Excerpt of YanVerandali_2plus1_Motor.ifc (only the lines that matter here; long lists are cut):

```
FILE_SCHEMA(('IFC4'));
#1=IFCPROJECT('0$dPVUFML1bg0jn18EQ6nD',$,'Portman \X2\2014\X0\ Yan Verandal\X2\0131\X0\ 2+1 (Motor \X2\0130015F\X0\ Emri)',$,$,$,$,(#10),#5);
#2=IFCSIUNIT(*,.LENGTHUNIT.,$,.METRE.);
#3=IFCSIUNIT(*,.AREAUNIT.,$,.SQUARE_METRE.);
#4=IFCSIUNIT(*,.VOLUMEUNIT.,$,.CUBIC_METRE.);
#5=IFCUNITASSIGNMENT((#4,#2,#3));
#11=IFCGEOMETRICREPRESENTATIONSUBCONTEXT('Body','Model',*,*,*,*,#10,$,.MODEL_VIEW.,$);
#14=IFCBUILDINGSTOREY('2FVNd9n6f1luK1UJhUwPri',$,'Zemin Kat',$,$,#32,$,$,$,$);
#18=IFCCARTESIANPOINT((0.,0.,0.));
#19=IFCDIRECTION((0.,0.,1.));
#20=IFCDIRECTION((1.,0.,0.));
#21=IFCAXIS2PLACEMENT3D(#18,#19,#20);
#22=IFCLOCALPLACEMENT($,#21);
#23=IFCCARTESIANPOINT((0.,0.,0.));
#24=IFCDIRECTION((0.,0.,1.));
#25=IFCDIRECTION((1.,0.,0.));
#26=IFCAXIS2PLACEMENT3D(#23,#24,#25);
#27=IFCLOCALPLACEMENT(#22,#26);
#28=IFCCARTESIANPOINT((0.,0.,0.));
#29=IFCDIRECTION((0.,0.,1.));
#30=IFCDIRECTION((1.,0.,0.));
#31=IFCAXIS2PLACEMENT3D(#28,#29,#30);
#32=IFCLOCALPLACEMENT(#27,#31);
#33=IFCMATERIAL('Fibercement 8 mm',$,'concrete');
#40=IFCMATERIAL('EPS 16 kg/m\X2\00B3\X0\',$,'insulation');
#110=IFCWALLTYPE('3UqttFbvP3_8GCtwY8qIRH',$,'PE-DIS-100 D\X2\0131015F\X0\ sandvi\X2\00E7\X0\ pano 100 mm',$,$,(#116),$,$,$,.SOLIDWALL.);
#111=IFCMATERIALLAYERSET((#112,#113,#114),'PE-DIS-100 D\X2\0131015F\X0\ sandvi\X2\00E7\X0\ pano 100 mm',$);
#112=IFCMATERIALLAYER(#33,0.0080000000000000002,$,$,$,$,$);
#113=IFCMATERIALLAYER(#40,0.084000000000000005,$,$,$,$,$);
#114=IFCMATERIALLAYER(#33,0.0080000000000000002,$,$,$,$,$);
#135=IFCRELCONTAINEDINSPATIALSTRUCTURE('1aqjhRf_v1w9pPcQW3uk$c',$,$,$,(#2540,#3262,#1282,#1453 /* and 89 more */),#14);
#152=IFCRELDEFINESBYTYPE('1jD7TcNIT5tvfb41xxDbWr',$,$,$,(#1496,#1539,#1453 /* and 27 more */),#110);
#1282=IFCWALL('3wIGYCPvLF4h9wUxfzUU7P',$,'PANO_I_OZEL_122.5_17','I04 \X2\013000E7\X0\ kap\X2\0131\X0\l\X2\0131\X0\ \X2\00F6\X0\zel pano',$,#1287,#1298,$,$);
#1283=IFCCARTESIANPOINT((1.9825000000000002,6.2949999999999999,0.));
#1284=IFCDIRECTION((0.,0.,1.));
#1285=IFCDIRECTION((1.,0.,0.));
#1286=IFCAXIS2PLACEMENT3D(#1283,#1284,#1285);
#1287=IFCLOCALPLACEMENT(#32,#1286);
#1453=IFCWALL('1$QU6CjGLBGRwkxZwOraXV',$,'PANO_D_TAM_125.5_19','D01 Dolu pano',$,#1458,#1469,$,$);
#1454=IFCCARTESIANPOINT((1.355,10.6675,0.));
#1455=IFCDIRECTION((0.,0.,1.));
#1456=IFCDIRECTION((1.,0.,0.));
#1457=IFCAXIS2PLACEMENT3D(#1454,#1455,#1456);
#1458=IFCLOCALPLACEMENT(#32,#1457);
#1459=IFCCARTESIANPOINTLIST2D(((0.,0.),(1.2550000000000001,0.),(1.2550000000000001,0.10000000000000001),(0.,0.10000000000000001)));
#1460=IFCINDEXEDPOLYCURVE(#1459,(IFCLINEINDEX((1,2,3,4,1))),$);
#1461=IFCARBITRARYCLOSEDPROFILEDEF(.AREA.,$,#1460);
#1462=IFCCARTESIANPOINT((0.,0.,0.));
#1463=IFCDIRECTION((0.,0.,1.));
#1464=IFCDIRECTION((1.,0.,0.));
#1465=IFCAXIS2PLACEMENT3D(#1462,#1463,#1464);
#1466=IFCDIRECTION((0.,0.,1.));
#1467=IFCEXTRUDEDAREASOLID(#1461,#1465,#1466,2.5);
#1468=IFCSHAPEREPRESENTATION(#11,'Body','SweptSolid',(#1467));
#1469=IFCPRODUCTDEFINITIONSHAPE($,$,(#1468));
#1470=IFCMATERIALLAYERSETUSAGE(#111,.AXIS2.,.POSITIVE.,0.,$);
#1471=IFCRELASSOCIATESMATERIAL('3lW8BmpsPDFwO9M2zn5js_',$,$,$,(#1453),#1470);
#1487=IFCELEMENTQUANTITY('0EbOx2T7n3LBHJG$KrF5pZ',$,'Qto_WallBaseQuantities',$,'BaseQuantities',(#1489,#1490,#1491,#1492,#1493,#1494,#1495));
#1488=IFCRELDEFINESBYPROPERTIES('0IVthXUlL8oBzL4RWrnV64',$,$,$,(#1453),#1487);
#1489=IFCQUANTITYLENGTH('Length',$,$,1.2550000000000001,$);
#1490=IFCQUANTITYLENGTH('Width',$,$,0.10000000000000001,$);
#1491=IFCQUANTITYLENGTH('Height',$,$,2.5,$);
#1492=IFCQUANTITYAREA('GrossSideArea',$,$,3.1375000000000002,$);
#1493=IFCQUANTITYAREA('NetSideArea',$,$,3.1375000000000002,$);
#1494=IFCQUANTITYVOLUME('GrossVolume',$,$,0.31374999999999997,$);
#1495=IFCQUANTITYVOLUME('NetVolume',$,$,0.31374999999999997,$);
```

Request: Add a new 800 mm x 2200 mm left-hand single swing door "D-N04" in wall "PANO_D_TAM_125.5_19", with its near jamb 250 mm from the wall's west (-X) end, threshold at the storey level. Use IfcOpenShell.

```python
import numpy as np
import ifcopenshell
import ifcopenshell.api.feature
import ifcopenshell.api.geometry
import ifcopenshell.api.pset
import ifcopenshell.api.root
import ifcopenshell.api.spatial
import ifcopenshell.geom
import ifcopenshell.util.element
import ifcopenshell.util.placement
import ifcopenshell.util.representation
import ifcopenshell.util.shape
import ifcopenshell.util.unit

model = ifcopenshell.open("YanVerandali_2plus1_Motor.ifc")
unit_scale = ifcopenshell.util.unit.calculate_unit_scale(model)
area_scale = ifcopenshell.util.unit.calculate_unit_scale(model, "AREAUNIT")
volume_scale = ifcopenshell.util.unit.calculate_unit_scale(model, "VOLUMEUNIT")
settings = ifcopenshell.geom.settings()


def volume(element):
    """Net volume in cubic metres, openings subtracted."""
    shape = ifcopenshell.geom.create_shape(settings, element)
    return ifcopenshell.util.shape.get_volume(shape.geometry)


wall = model.by_guid("1$QU6CjGLBGRwkxZwOraXV")
storey = ifcopenshell.util.element.get_container(wall, ifc_class="IfcBuildingStorey")
context = ifcopenshell.util.representation.get_context(model, "Model", "Body", "MODEL_VIEW")
before = volume(wall)

width, height, from_end, sill = 0.8, 2.2, 0.25, 0.0  # metres

# The wall runs along its own X axis, and the end named is its -X end.
wall_shape = ifcopenshell.geom.create_shape(settings, wall)
x, y, z = ifcopenshell.util.shape.get_vertices(wall_shape.geometry).T
start = x.min() + from_end
face, thickness = float(y.min()), float(y.max() - y.min())
wall_matrix = ifcopenshell.util.placement.get_local_placement(wall.ObjectPlacement)
level = ifcopenshell.util.placement.get_local_placement(storey.ObjectPlacement)[2, 3]


def in_wall(x, y):
    """Placement at x, y metres in the wall's axes, at sill height."""
    matrix = wall_matrix.copy()
    matrix[:, 3] = wall_matrix @ np.array([x / unit_scale, y / unit_scale, 0.0, 1.0])
    matrix[2, 3] = level + sill / unit_scale
    return matrix


# Opening: a box that overshoots both wall faces by 50 mm.
opening = ifcopenshell.api.root.create_entity(model, ifc_class="IfcOpeningElement", predefined_type="OPENING")
box = ifcopenshell.api.geometry.add_wall_representation(
    model, context=context, length=width, height=height, thickness=thickness + 0.1
)
ifcopenshell.api.geometry.assign_representation(model, product=opening, representation=box)
ifcopenshell.api.geometry.edit_object_placement(model, product=opening, matrix=in_wall(start, face - 0.05), is_si=False)
ifcopenshell.api.feature.add_feature(model, feature=opening, element=wall)

door = ifcopenshell.api.root.create_entity(model, ifc_class="IfcDoor", name="D-N04", predefined_type="DOOR")
door.OverallWidth, door.OverallHeight = width / unit_scale, height / unit_scale
door.OperationType = "SINGLE_SWING_LEFT"
body = ifcopenshell.api.geometry.add_door_representation(
    model,
    context=context,
    overall_width=door.OverallWidth,
    overall_height=door.OverallHeight,
    operation_type="SINGLE_SWING_LEFT",
    lining_properties={"LiningDepth": thickness / unit_scale, "ThresholdDepth": thickness / unit_scale},
)
ifcopenshell.api.geometry.assign_representation(model, product=door, representation=body)
ifcopenshell.api.spatial.assign_container(model, products=[door], relating_structure=storey)
ifcopenshell.api.feature.add_filling(model, opening=opening, element=door)

# The lining spans the wall, so the door starts at the wall face.
ifcopenshell.api.geometry.edit_object_placement(model, product=door, matrix=in_wall(start, face), is_si=False)

after = volume(wall)

# Update the wall's stored quantities.
qto = model.by_id(ifcopenshell.util.element.get_pset(wall, "Qto_WallBaseQuantities", should_inherit=False)["id"])
ifcopenshell.api.pset.edit_qto(model, qto=qto, properties={
    "NetSideArea": after / thickness / area_scale,
    "NetVolume": after / volume_scale,
})

print(f"wall volume {before:.3f} -> {after:.3f} m3")

model.write("YanVerandali_2plus1_Motor-out.ifc")
```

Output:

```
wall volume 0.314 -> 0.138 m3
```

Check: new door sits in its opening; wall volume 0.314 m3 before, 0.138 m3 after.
